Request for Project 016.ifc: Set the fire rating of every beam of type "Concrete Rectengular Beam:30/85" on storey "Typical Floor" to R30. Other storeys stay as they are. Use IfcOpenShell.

First a look at what the model holds.

```python
import ifcopenshell
import ifcopenshell.util.element

model = ifcopenshell.open("Project 016.ifc")
print(model.schema)
storey = next(s for s in model.by_type("IfcBuildingStorey") if s.Name == "Typical Floor")
beams = [e for e in ifcopenshell.util.element.get_decomposition(storey) if e.is_a("IfcBeam")]
seen = {}
for e in beams:
    element_type = ifcopenshell.util.element.get_type(e)
    key = (element_type.Name if element_type != e and element_type else None, ifcopenshell.util.element.get_pset(e, "Pset_BeamCommon", "FireRating"))
    seen[key] = seen.get(key, 0) + 1
for (name, value), count in sorted(seen.items(), key=str):
    print(count, "x", name, "|", value)
```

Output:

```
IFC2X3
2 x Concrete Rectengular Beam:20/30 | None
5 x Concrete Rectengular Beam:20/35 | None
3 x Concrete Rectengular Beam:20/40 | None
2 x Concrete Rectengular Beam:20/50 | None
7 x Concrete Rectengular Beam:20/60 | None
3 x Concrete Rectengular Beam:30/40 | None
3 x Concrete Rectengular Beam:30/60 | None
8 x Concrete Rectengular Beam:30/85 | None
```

```python
import ifcopenshell
import ifcopenshell.api.pset
import ifcopenshell.util.element

model = ifcopenshell.open("Project 016.ifc")

storey = next(s for s in model.by_type("IfcBuildingStorey") if s.Name == "Typical Floor")
beams = [e for e in ifcopenshell.util.element.get_decomposition(storey) if e.is_a("IfcBeam")]

count = 0
for e in beams:
    element_type = ifcopenshell.util.element.get_type(e)
    if element_type in (None, e) or element_type.Name != "Concrete Rectengular Beam:30/85":
        continue
    # add_pset returns the element's existing set when there is one.
    pset = ifcopenshell.api.pset.add_pset(model, product=e, name="Pset_BeamCommon")
    ifcopenshell.api.pset.edit_pset(model, pset=pset, properties={"FireRating": "R30"})
    count += 1

print(count, "beams updated")

model.write("Project 016_edited.ifc")
```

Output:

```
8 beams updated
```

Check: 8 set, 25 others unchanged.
